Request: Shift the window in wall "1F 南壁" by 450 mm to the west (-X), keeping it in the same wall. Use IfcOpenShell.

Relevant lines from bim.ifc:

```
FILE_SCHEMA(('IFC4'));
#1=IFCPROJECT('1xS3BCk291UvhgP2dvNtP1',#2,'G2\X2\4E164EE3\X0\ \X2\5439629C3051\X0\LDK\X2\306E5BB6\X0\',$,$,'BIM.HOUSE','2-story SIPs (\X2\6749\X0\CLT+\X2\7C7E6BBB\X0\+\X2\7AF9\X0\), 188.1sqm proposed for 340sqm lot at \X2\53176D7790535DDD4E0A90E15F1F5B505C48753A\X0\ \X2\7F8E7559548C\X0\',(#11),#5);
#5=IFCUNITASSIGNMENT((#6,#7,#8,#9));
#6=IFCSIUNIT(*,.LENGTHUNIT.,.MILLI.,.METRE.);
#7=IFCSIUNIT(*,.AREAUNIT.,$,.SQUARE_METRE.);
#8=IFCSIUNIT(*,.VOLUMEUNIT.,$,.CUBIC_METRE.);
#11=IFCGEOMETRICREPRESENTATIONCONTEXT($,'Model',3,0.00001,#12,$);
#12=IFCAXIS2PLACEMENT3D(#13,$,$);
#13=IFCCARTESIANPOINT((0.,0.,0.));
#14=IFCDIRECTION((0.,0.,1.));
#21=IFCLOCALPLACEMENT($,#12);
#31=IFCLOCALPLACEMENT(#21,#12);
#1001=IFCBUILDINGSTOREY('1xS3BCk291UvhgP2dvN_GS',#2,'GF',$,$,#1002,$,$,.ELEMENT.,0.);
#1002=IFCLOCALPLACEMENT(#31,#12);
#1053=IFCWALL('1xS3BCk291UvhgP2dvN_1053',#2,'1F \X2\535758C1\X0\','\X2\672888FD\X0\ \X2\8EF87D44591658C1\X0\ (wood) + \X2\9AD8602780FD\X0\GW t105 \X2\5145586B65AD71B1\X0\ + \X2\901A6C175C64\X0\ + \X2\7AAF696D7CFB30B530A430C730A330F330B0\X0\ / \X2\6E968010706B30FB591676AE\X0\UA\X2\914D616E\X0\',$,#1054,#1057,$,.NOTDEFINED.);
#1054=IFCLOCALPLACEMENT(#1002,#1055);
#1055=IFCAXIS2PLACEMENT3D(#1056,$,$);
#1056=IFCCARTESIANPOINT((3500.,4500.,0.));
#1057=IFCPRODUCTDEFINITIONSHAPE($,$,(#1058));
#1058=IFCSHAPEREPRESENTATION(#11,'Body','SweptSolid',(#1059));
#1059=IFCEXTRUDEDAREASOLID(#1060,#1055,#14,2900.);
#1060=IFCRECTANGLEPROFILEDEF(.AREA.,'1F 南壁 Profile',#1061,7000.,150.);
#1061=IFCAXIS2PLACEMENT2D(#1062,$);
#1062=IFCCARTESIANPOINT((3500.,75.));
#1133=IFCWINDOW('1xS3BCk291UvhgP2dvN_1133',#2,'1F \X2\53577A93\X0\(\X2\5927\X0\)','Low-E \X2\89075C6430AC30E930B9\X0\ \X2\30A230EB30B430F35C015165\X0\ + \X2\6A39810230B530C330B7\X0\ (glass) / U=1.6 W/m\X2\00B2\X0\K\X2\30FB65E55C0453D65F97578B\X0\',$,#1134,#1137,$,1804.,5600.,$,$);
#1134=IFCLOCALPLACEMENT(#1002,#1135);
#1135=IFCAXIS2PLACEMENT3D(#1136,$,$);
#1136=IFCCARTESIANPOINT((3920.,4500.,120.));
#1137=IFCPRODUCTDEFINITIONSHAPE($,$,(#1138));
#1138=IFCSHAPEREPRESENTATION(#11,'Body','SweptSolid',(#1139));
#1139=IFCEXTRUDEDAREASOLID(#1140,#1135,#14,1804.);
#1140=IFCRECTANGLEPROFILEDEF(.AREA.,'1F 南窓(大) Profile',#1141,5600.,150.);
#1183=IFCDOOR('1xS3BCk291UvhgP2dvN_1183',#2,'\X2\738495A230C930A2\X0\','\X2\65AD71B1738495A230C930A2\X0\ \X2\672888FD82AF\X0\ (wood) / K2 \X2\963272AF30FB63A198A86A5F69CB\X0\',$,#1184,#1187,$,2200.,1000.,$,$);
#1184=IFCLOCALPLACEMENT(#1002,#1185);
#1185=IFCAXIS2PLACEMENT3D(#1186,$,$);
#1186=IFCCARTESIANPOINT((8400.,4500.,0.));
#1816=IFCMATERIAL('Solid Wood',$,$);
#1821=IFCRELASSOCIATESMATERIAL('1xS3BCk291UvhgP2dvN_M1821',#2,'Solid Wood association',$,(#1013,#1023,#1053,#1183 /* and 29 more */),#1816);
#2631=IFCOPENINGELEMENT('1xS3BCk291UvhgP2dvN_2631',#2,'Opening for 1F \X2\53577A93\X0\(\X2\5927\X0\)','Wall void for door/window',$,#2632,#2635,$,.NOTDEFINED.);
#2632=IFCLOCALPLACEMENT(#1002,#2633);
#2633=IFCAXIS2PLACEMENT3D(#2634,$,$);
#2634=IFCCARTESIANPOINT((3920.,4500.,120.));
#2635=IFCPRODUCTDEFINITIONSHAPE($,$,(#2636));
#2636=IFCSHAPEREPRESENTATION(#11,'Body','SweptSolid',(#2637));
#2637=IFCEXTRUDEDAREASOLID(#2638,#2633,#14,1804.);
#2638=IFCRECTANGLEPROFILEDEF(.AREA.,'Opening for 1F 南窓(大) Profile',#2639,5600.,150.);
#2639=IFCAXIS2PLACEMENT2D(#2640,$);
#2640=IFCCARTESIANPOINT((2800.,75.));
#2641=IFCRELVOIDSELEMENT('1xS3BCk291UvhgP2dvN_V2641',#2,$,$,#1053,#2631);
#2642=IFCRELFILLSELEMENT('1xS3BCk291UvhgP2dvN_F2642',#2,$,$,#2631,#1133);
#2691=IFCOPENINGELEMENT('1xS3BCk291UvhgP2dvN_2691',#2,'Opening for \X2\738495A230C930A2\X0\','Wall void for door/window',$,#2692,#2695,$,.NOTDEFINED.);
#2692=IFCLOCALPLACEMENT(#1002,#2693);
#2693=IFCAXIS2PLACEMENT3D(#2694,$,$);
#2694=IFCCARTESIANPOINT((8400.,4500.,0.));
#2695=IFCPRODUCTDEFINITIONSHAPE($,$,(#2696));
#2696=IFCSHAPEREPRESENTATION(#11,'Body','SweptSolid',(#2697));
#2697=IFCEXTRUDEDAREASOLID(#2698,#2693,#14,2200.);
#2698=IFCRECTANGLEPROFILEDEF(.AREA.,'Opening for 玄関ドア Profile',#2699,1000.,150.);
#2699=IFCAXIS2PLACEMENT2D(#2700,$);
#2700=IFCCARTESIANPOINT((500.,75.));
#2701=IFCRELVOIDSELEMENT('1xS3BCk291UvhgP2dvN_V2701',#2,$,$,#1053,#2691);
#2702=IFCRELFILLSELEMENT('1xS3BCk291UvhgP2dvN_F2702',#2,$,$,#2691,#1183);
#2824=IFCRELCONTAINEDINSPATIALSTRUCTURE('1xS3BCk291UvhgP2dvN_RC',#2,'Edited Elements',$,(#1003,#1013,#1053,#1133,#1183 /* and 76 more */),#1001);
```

```python
import ifcopenshell
import ifcopenshell.api.geometry
import ifcopenshell.util.placement

model = ifcopenshell.open("bim.ifc")

window = model.by_guid("1xS3BCk291UvhgP2dvN_1133")
opening = window.FillsVoids[0].RelatingOpeningElement
wall = opening.VoidsElements[0].RelatingBuildingElement

wall_matrix = ifcopenshell.util.placement.get_local_placement(wall.ObjectPlacement)
shift = wall_matrix[:3, 0] * -450.0
before = ifcopenshell.util.placement.get_local_placement(window.ObjectPlacement)[:3, 3].copy()

# The window is not placed relative to its opening, so move both.
for product in (opening, window):
    matrix = ifcopenshell.util.placement.get_local_placement(product.ObjectPlacement)
    matrix[:3, 3] += shift
    ifcopenshell.api.geometry.edit_object_placement(model, product=product, matrix=matrix, is_si=False)

after = ifcopenshell.util.placement.get_local_placement(window.ObjectPlacement)[:3, 3]
print("window moved by", (after - before).round(3) + 0.0)

model.write("bim_edited.ifc")
```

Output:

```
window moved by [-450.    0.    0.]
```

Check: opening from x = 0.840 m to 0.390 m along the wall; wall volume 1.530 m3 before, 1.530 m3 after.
